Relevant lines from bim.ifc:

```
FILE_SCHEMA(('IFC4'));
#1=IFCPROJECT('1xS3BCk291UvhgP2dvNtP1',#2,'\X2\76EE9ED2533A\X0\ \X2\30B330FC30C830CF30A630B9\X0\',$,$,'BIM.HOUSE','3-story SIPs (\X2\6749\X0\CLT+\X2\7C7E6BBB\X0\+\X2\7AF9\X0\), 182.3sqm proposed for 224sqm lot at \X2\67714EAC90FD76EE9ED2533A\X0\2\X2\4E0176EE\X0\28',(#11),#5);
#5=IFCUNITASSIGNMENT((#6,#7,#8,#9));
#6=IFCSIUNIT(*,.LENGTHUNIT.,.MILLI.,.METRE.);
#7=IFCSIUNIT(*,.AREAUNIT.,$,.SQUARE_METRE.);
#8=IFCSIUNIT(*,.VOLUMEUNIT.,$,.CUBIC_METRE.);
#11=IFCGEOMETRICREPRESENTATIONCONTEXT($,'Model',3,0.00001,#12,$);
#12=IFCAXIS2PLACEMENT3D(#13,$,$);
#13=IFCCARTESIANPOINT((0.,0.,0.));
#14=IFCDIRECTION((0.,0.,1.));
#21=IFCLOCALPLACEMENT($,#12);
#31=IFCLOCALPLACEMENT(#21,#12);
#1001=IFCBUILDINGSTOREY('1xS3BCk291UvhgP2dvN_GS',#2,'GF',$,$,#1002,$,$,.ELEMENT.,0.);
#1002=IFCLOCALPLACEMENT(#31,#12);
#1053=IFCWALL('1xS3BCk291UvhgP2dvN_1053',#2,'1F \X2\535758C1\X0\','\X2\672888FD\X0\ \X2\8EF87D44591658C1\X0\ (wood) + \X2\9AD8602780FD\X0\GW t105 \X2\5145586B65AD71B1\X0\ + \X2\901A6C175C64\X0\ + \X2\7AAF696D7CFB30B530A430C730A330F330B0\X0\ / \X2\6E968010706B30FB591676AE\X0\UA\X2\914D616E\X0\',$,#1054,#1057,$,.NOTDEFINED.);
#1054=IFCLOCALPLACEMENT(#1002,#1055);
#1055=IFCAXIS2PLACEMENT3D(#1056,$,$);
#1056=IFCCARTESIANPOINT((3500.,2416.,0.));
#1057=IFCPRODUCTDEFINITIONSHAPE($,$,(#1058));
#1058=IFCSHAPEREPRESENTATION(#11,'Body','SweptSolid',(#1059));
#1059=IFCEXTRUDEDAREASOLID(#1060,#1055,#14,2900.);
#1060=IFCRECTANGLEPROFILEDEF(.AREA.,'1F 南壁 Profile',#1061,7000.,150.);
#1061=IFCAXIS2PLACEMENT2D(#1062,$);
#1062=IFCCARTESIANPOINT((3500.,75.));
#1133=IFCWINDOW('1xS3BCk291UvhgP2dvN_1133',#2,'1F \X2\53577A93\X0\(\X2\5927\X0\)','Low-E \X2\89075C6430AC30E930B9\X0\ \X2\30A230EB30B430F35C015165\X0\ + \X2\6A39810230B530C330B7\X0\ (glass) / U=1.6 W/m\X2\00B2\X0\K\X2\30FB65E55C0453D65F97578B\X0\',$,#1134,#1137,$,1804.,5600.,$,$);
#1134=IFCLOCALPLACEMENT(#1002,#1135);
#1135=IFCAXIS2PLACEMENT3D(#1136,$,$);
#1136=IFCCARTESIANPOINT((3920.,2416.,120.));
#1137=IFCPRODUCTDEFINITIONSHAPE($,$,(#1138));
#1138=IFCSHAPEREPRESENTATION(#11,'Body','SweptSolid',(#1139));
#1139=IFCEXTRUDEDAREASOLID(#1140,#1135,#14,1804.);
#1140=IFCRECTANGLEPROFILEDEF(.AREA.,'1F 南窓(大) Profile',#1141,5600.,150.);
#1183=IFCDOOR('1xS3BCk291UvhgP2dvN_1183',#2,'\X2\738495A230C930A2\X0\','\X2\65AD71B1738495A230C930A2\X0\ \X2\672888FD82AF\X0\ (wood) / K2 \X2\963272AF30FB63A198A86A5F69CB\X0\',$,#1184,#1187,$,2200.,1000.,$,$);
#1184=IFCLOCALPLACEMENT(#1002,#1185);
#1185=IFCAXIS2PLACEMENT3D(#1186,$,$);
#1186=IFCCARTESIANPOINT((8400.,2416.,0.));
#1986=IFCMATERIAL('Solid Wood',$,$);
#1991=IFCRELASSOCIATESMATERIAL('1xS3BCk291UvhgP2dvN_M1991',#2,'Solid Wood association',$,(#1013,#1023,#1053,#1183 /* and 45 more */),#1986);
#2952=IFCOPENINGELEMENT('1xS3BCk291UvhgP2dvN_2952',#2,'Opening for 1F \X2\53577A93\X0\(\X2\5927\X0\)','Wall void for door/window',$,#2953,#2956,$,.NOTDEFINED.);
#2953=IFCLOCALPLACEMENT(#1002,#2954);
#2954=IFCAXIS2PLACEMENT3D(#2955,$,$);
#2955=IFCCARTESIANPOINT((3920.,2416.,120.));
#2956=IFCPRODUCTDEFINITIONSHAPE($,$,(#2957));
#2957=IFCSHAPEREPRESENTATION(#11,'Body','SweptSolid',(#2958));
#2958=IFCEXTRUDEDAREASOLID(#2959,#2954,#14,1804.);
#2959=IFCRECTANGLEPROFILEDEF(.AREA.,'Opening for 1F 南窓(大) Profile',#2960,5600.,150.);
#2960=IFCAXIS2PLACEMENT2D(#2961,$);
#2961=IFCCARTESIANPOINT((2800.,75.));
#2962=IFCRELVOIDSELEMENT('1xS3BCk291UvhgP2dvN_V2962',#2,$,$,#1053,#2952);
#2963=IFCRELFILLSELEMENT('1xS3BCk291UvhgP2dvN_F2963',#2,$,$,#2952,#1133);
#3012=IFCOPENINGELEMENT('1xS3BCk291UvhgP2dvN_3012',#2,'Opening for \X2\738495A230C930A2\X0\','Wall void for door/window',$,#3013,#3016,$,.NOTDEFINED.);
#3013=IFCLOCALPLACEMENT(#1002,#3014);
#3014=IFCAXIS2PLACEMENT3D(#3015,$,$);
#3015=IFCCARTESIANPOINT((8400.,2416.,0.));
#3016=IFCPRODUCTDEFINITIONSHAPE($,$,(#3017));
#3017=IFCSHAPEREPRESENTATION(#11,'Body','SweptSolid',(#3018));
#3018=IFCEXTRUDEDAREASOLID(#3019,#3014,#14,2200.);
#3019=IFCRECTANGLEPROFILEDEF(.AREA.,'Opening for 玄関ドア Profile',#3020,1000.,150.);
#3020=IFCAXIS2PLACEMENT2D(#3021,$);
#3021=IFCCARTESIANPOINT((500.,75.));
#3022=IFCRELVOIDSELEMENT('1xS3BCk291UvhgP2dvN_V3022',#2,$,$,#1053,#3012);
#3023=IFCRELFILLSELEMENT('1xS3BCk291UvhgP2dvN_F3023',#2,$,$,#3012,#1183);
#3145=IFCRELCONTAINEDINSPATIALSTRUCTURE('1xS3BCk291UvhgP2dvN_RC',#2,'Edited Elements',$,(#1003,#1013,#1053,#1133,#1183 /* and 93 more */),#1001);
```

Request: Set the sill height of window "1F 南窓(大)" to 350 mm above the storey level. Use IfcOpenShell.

```python
import numpy as np
import ifcopenshell
import ifcopenshell.api.geometry
import ifcopenshell.geom
import ifcopenshell.util.element
import ifcopenshell.util.placement
import ifcopenshell.util.shape
import ifcopenshell.util.unit

model = ifcopenshell.open("bim.ifc")
unit_scale = ifcopenshell.util.unit.calculate_unit_scale(model)

window = model.by_guid("1xS3BCk291UvhgP2dvN_1133")
opening = window.FillsVoids[0].RelatingOpeningElement
storey = ifcopenshell.util.element.get_container(window, ifc_class="IfcBuildingStorey")
level = ifcopenshell.util.placement.get_local_placement(storey.ObjectPlacement)[2, 3]

# The opening's origin need not be at the sill, so measure its lowest point.
shape = ifcopenshell.geom.create_shape(ifcopenshell.geom.settings(), opening)
bottom = ifcopenshell.util.shape.get_shape_bottom_elevation(shape, shape.geometry) / unit_scale
dz = level + 350.0 - bottom

shift = np.array([0.0, 0.0, dz])
# The window is not placed relative to its opening, so move both.
for product in (opening, window):
    matrix = ifcopenshell.util.placement.get_local_placement(product.ObjectPlacement)
    matrix[:3, 3] += shift
    ifcopenshell.api.geometry.edit_object_placement(model, product=product, matrix=matrix, is_si=False)

print(f"moved by {dz * unit_scale:+.3f} m")

model.write("bim_updated.ifc")
```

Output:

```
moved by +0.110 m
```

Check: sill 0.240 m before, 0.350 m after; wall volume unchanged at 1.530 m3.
